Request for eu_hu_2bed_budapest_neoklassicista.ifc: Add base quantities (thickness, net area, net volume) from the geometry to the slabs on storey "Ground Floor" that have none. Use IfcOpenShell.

First a look at what the model holds.

```python
import ifcopenshell
import ifcopenshell.util.element
import ifcopenshell.util.unit

model = ifcopenshell.open("eu_hu_2bed_budapest_neoklassicista.ifc")
print(model.schema)
for unit_type in ("LENGTHUNIT", "AREAUNIT", "VOLUMEUNIT"):
    print(unit_type, ifcopenshell.util.unit.calculate_unit_scale(model, unit_type))
storey = next(s for s in model.by_type("IfcBuildingStorey") if s.Name == "Ground Floor")
slabs = [e for e in ifcopenshell.util.element.get_decomposition(storey) if e.is_a("IfcSlab")]
for e in sorted(slabs, key=lambda e: e.id()):
    print(e.id(), e.is_a(), e.Name, list(ifcopenshell.util.element.get_psets(e, qtos_only=True)), sep=" | ")
```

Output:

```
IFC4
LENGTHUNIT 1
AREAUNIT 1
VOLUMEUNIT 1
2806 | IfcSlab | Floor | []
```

```python
import ifcopenshell
import ifcopenshell.api.pset
import ifcopenshell.geom
import ifcopenshell.util.element
import ifcopenshell.util.shape
import ifcopenshell.util.unit

model = ifcopenshell.open("eu_hu_2bed_budapest_neoklassicista.ifc")
unit_scale = ifcopenshell.util.unit.calculate_unit_scale(model)
area_scale = ifcopenshell.util.unit.calculate_unit_scale(model, "AREAUNIT")
volume_scale = ifcopenshell.util.unit.calculate_unit_scale(model, "VOLUMEUNIT")
settings = ifcopenshell.geom.settings()

storey = next(s for s in model.by_type("IfcBuildingStorey") if s.Name == "Ground Floor")
slabs = [e for e in ifcopenshell.util.element.get_decomposition(storey) if e.is_a("IfcSlab")]

for e in sorted(slabs, key=lambda e: e.id()):
    if ifcopenshell.util.element.get_psets(e, qtos_only=True, should_inherit=False):
        continue
    # Geometry comes back in metres, in the element's own axes.
    shape = ifcopenshell.geom.create_shape(settings, e)
    values = {
        "Width": ifcopenshell.util.shape.get_z(shape.geometry) / unit_scale,
        "NetArea": ifcopenshell.util.shape.get_footprint_area(shape.geometry) / area_scale,
        "NetVolume": ifcopenshell.util.shape.get_volume(shape.geometry) / volume_scale,
    }
    qto = ifcopenshell.api.pset.add_qto(model, product=e, name="Qto_SlabBaseQuantities")
    ifcopenshell.api.pset.edit_qto(model, qto=qto, properties=values)
    print(e.id(), {k: round(v, 3) for k, v in values.items()})

model.write("eu_hu_2bed_budapest_neoklassicista_v2.ifc")
```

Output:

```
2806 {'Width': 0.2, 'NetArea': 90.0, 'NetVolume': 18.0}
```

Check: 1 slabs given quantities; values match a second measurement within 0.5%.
